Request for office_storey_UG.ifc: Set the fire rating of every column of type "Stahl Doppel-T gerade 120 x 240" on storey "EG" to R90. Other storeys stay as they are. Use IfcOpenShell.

First a look at what the model holds.

```python
import ifcopenshell
import ifcopenshell.util.element

model = ifcopenshell.open("office_storey_UG.ifc")
print(model.schema)
storey = next(s for s in model.by_type("IfcBuildingStorey") if s.Name == "EG")
columns = [e for e in ifcopenshell.util.element.get_decomposition(storey) if e.is_a("IfcColumn")]
seen = {}
for e in columns:
    element_type = ifcopenshell.util.element.get_type(e)
    key = (element_type.Name if element_type != e and element_type else None, ifcopenshell.util.element.get_pset(e, "Pset_ColumnCommon", "FireRating"))
    seen[key] = seen.get(key, 0) + 1
for (name, value), count in sorted(seen.items(), key=str):
    print(count, "x", name, "|", value)
```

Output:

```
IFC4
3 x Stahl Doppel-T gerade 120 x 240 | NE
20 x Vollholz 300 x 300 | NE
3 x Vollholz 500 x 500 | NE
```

```python
import ifcopenshell
import ifcopenshell.api.pset
import ifcopenshell.util.element

model = ifcopenshell.open("office_storey_UG.ifc")

storey = next(s for s in model.by_type("IfcBuildingStorey") if s.Name == "EG")
columns = [e for e in ifcopenshell.util.element.get_decomposition(storey) if e.is_a("IfcColumn")]

count = 0
for e in columns:
    element_type = ifcopenshell.util.element.get_type(e)
    if element_type in (None, e) or element_type.Name != "Stahl Doppel-T gerade 120 x 240":
        continue
    # add_pset returns the element's existing set when there is one.
    pset = ifcopenshell.api.pset.add_pset(model, product=e, name="Pset_ColumnCommon")
    ifcopenshell.api.pset.edit_pset(model, pset=pset, properties={"FireRating": "R90"})
    count += 1

print(count, "columns updated")

model.write("office_storey_UG-out.ifc")
```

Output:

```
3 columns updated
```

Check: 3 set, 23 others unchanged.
